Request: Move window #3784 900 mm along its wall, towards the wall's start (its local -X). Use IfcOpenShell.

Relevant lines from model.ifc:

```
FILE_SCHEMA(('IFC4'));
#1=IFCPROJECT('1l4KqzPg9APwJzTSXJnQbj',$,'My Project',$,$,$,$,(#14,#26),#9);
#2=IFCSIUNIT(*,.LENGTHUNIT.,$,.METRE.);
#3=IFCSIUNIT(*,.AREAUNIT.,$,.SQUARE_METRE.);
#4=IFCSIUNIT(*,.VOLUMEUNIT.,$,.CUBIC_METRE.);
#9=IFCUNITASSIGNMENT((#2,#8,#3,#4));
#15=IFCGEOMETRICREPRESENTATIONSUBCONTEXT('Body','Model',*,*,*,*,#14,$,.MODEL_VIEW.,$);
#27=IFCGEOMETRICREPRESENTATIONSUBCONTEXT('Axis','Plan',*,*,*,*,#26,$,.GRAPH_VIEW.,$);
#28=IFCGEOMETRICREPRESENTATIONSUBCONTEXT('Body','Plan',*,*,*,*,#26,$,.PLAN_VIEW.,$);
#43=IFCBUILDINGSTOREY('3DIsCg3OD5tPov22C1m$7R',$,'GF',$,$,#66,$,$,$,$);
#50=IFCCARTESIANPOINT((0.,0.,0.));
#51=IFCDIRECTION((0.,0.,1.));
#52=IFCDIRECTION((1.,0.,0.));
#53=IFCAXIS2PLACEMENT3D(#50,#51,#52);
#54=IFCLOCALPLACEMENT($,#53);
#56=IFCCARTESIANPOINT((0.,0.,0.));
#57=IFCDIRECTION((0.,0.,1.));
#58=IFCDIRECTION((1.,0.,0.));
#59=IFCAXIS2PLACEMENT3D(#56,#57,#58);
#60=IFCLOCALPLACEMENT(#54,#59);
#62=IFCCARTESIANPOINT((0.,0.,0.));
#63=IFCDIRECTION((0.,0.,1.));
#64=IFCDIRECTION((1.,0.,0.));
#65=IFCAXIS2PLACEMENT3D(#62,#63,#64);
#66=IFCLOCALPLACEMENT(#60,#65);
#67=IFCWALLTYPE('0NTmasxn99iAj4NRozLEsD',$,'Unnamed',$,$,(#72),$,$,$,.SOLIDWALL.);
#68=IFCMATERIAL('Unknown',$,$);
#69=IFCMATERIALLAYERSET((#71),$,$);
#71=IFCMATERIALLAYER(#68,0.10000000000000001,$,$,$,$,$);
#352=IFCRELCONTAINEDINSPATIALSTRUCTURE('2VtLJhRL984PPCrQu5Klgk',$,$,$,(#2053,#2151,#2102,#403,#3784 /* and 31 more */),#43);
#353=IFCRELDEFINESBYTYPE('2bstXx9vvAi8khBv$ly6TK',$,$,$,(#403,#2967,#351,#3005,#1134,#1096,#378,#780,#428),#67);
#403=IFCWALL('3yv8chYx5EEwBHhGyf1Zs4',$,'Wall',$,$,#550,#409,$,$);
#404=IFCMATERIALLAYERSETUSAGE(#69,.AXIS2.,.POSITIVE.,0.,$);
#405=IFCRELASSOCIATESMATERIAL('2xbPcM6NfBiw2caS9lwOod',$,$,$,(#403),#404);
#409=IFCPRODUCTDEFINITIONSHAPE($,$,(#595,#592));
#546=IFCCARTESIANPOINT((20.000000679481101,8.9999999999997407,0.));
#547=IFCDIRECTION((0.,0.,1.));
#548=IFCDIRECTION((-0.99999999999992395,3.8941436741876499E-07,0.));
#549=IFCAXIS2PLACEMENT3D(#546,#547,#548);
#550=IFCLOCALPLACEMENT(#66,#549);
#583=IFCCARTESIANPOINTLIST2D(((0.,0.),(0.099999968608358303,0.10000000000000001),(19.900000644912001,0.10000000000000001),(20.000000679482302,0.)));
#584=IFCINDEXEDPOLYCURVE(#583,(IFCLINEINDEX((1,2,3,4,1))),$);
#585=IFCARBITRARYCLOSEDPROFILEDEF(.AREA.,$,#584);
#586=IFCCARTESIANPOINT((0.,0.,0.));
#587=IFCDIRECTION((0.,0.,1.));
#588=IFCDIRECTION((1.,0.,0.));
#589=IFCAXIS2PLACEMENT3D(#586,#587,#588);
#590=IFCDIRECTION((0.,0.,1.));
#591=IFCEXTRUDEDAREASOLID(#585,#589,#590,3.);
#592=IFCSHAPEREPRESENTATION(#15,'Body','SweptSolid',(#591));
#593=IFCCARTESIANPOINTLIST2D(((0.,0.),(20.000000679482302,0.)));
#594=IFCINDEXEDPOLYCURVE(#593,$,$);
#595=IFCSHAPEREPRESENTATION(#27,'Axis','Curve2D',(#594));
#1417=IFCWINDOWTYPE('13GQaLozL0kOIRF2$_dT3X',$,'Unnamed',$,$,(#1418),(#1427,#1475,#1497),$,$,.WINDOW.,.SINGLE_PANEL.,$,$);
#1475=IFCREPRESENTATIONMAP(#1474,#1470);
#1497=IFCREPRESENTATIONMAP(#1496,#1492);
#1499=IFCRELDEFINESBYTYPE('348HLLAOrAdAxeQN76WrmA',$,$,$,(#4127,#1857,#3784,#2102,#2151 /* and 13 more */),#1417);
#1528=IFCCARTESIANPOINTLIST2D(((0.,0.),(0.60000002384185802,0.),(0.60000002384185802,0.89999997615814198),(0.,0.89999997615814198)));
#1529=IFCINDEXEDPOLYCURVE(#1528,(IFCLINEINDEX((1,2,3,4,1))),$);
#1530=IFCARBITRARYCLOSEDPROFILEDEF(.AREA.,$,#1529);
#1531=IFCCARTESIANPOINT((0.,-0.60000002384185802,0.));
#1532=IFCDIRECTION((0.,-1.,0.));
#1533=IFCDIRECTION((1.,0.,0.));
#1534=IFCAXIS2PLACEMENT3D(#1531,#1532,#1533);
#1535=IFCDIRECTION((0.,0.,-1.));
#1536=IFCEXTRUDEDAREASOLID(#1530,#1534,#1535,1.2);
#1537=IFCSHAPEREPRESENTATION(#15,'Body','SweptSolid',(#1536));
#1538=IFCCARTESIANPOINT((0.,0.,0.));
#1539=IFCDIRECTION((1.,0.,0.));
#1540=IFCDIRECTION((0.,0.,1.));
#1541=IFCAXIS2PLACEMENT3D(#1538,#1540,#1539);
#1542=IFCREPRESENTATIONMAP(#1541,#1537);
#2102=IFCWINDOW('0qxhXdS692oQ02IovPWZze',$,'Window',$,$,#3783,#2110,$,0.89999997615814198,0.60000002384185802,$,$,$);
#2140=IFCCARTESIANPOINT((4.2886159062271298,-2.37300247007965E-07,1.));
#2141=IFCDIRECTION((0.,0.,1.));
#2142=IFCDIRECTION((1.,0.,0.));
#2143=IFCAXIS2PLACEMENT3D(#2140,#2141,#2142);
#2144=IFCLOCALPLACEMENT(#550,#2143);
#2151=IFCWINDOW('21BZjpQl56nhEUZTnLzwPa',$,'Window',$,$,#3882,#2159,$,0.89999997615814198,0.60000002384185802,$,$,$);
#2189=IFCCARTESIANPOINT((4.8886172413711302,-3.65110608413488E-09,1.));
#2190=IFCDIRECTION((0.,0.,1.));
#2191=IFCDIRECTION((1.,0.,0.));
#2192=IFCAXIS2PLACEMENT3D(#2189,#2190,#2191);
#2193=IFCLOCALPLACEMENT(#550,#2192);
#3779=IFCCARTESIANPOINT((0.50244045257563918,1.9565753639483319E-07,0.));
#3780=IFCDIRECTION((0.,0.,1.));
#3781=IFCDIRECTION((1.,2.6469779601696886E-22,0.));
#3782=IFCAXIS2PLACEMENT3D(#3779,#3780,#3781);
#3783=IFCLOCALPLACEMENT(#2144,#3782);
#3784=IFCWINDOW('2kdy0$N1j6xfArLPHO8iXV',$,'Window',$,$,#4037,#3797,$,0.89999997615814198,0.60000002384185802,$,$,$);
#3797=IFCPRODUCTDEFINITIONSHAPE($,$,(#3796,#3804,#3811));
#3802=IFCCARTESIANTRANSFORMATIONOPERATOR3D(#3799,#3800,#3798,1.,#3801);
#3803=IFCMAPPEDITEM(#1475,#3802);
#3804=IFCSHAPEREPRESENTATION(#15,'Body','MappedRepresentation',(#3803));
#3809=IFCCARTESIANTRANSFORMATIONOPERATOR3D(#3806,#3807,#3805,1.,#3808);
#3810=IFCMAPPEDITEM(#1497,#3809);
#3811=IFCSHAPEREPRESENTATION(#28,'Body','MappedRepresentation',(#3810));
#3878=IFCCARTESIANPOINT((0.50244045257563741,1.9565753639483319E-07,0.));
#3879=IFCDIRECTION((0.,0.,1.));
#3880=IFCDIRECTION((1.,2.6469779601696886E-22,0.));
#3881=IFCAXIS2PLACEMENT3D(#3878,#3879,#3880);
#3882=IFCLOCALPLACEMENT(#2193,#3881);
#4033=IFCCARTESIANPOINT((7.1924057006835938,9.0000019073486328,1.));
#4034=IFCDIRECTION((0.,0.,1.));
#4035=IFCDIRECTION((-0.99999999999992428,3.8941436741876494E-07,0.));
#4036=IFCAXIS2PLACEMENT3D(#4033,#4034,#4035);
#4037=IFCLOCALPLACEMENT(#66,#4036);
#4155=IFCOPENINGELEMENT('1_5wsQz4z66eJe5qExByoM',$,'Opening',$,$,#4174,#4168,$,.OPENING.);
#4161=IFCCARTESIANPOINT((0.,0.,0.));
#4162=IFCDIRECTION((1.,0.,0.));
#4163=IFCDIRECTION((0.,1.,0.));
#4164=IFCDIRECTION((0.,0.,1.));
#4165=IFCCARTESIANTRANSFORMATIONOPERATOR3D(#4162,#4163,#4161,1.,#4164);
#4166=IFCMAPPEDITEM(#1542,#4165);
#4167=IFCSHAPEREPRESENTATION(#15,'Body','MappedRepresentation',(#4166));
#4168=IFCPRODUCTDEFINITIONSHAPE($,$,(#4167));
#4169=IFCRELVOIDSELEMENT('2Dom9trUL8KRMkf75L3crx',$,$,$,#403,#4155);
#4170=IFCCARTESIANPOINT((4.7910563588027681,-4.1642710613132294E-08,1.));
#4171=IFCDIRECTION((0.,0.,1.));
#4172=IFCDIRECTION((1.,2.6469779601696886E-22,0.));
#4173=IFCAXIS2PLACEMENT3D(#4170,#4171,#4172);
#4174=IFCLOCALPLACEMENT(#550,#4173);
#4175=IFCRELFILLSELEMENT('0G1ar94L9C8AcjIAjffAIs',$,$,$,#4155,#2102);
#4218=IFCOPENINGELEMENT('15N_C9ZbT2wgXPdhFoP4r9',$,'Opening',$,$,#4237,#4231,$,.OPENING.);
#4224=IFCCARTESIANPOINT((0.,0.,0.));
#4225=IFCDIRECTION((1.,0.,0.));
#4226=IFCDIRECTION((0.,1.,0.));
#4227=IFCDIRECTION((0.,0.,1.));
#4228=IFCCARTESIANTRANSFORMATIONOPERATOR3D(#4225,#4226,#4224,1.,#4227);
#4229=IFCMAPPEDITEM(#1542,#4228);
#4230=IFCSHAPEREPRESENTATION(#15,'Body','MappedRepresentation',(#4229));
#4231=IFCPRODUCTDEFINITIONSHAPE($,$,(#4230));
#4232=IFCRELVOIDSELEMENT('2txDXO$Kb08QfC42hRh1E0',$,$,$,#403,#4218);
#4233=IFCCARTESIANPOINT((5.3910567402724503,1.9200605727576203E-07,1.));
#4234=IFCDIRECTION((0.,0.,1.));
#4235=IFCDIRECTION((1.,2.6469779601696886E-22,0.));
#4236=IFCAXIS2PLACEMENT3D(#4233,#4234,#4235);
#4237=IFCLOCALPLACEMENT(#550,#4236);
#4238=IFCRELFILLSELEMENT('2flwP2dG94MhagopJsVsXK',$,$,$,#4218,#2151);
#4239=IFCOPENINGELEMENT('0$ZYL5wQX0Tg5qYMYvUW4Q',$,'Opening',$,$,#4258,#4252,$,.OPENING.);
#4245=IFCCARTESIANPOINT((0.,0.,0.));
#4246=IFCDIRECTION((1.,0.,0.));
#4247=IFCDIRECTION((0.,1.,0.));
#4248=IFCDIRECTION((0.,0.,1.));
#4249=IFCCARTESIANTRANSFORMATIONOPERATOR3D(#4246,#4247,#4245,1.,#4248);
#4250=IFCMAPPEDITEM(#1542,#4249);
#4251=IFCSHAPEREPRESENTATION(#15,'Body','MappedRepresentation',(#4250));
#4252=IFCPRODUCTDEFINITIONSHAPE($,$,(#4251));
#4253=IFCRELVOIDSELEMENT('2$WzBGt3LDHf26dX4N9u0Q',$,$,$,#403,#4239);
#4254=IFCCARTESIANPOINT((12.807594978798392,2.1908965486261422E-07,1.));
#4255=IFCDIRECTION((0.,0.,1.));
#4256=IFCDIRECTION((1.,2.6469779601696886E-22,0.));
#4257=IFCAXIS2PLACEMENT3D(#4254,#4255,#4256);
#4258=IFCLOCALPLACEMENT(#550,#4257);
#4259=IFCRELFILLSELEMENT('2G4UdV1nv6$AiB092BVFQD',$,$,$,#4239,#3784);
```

```python
import ifcopenshell
import ifcopenshell.api.geometry
import ifcopenshell.util.placement
import ifcopenshell.util.unit

model = ifcopenshell.open("model.ifc")
unit_scale = ifcopenshell.util.unit.calculate_unit_scale(model)

window = model.by_id(3784)
opening = window.FillsVoids[0].RelatingOpeningElement
wall = opening.VoidsElements[0].RelatingBuildingElement

wall_matrix = ifcopenshell.util.placement.get_local_placement(wall.ObjectPlacement)
shift = wall_matrix[:3, 0] * -0.9 / unit_scale
before = ifcopenshell.util.placement.get_local_placement(window.ObjectPlacement)[:3, 3].copy()

# The window is not placed relative to its opening, so move both.
for product in (opening, window):
    matrix = ifcopenshell.util.placement.get_local_placement(product.ObjectPlacement)
    matrix[:3, 3] += shift
    ifcopenshell.api.geometry.edit_object_placement(model, product=product, matrix=matrix, is_si=False)

after = ifcopenshell.util.placement.get_local_placement(window.ObjectPlacement)[:3, 3]
print("window moved by", (after - before).round(3) + 0.0)

model.write("model_rev.ifc")
```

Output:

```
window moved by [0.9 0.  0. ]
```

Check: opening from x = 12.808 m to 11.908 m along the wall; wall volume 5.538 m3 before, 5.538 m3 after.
